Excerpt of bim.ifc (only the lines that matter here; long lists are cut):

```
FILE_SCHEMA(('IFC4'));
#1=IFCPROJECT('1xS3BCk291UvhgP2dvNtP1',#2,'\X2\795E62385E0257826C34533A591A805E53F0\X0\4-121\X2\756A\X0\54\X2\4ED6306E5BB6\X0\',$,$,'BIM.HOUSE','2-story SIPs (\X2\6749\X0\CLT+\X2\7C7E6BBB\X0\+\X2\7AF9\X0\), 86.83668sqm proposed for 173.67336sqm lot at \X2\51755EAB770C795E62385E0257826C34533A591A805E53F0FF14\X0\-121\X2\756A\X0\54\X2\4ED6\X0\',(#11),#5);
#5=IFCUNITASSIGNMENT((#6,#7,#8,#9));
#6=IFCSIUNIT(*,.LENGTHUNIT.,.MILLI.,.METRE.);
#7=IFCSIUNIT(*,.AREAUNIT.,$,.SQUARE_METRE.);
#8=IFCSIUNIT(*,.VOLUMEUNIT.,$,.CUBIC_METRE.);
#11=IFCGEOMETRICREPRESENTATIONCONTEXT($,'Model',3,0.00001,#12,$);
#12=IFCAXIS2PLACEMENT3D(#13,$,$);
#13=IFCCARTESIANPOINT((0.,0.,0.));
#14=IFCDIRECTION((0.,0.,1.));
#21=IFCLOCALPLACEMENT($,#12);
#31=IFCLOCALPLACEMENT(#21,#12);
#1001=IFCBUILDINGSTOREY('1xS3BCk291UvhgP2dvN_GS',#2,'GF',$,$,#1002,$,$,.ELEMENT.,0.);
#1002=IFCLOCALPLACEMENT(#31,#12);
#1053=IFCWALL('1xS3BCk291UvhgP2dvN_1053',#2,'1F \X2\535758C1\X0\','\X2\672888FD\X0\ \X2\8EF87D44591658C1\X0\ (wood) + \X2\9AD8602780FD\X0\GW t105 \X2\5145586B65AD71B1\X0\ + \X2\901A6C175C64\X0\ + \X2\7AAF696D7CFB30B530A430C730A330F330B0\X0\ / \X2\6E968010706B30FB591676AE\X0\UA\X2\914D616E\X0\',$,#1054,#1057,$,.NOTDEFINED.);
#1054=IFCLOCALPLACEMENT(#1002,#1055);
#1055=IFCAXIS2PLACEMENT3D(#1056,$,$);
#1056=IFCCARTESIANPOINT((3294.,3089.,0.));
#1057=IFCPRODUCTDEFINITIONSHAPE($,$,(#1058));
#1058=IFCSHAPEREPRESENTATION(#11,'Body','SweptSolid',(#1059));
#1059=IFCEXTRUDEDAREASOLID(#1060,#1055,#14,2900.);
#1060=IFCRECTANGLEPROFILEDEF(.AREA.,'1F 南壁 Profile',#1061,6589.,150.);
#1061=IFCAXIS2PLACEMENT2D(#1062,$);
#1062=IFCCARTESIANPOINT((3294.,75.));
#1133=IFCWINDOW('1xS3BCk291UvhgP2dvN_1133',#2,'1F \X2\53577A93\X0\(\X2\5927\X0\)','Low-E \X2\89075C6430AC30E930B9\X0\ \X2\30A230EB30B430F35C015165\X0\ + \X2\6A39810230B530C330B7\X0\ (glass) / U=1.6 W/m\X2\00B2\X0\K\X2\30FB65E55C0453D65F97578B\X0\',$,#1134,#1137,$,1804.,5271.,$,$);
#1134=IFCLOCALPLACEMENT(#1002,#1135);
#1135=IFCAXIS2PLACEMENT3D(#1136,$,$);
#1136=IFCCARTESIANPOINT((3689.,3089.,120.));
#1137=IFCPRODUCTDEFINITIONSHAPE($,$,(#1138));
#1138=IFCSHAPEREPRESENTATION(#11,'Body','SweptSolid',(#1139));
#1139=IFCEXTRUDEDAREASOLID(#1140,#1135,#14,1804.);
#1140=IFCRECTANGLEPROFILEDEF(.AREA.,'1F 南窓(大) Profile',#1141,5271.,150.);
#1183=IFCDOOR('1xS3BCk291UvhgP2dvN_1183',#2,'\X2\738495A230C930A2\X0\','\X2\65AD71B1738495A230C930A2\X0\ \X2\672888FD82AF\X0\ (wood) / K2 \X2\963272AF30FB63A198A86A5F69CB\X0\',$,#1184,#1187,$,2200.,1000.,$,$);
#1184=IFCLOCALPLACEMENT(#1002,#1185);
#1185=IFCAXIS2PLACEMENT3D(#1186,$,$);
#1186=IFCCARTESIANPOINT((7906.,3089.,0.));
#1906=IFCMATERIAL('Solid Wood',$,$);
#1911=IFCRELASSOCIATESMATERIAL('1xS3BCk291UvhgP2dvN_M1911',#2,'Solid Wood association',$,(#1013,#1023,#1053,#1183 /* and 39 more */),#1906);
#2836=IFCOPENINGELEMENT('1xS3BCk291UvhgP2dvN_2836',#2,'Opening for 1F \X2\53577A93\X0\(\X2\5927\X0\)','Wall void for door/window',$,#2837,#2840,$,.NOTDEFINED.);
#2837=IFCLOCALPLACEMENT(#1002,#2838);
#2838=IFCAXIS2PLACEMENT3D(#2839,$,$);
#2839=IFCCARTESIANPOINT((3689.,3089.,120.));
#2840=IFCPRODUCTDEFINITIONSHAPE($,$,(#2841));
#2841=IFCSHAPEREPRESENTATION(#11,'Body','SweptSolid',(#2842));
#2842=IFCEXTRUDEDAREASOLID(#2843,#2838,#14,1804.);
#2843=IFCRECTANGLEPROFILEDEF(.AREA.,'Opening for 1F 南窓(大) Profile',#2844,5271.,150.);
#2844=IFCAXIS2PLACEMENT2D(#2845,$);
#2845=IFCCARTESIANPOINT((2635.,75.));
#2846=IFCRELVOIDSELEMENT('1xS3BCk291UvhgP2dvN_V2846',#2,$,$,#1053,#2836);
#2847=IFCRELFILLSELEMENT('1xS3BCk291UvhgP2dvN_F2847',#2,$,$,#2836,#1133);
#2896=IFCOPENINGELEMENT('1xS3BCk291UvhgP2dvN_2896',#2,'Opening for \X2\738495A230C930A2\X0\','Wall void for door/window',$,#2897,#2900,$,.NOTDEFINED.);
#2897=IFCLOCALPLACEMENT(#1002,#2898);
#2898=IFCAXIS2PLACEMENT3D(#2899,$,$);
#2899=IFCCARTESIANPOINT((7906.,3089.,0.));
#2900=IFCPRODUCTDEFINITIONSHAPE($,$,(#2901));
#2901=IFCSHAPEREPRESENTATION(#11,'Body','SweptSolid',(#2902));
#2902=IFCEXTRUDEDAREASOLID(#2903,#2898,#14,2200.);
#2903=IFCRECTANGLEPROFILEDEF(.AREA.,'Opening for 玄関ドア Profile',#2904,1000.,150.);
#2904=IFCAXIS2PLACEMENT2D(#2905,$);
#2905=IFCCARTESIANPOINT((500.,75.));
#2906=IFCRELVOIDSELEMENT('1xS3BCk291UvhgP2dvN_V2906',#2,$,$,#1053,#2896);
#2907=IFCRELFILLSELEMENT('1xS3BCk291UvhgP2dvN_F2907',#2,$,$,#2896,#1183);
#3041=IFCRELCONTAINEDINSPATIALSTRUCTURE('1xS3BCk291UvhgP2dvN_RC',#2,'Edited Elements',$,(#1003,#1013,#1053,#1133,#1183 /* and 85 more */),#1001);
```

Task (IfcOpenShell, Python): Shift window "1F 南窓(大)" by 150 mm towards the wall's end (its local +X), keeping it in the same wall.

```python
import ifcopenshell
import ifcopenshell.api.geometry
import ifcopenshell.util.placement

model = ifcopenshell.open("bim.ifc")

window = model.by_id(1133)
opening = window.FillsVoids[0].RelatingOpeningElement
wall = opening.VoidsElements[0].RelatingBuildingElement

wall_matrix = ifcopenshell.util.placement.get_local_placement(wall.ObjectPlacement)
shift = wall_matrix[:3, 0] * 150.0
before = ifcopenshell.util.placement.get_local_placement(window.ObjectPlacement)[:3, 3].copy()

# The window is not placed relative to its opening, so move both.
for product in (opening, window):
    matrix = ifcopenshell.util.placement.get_local_placement(product.ObjectPlacement)
    matrix[:3, 3] += shift
    ifcopenshell.api.geometry.edit_object_placement(model, product=product, matrix=matrix, is_si=False)

after = ifcopenshell.util.placement.get_local_placement(window.ObjectPlacement)[:3, 3]
print("window moved by", (after - before).round(3) + 0.0)

model.write("bim_rev.ifc")
```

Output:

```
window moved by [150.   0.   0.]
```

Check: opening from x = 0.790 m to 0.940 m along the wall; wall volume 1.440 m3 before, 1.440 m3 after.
